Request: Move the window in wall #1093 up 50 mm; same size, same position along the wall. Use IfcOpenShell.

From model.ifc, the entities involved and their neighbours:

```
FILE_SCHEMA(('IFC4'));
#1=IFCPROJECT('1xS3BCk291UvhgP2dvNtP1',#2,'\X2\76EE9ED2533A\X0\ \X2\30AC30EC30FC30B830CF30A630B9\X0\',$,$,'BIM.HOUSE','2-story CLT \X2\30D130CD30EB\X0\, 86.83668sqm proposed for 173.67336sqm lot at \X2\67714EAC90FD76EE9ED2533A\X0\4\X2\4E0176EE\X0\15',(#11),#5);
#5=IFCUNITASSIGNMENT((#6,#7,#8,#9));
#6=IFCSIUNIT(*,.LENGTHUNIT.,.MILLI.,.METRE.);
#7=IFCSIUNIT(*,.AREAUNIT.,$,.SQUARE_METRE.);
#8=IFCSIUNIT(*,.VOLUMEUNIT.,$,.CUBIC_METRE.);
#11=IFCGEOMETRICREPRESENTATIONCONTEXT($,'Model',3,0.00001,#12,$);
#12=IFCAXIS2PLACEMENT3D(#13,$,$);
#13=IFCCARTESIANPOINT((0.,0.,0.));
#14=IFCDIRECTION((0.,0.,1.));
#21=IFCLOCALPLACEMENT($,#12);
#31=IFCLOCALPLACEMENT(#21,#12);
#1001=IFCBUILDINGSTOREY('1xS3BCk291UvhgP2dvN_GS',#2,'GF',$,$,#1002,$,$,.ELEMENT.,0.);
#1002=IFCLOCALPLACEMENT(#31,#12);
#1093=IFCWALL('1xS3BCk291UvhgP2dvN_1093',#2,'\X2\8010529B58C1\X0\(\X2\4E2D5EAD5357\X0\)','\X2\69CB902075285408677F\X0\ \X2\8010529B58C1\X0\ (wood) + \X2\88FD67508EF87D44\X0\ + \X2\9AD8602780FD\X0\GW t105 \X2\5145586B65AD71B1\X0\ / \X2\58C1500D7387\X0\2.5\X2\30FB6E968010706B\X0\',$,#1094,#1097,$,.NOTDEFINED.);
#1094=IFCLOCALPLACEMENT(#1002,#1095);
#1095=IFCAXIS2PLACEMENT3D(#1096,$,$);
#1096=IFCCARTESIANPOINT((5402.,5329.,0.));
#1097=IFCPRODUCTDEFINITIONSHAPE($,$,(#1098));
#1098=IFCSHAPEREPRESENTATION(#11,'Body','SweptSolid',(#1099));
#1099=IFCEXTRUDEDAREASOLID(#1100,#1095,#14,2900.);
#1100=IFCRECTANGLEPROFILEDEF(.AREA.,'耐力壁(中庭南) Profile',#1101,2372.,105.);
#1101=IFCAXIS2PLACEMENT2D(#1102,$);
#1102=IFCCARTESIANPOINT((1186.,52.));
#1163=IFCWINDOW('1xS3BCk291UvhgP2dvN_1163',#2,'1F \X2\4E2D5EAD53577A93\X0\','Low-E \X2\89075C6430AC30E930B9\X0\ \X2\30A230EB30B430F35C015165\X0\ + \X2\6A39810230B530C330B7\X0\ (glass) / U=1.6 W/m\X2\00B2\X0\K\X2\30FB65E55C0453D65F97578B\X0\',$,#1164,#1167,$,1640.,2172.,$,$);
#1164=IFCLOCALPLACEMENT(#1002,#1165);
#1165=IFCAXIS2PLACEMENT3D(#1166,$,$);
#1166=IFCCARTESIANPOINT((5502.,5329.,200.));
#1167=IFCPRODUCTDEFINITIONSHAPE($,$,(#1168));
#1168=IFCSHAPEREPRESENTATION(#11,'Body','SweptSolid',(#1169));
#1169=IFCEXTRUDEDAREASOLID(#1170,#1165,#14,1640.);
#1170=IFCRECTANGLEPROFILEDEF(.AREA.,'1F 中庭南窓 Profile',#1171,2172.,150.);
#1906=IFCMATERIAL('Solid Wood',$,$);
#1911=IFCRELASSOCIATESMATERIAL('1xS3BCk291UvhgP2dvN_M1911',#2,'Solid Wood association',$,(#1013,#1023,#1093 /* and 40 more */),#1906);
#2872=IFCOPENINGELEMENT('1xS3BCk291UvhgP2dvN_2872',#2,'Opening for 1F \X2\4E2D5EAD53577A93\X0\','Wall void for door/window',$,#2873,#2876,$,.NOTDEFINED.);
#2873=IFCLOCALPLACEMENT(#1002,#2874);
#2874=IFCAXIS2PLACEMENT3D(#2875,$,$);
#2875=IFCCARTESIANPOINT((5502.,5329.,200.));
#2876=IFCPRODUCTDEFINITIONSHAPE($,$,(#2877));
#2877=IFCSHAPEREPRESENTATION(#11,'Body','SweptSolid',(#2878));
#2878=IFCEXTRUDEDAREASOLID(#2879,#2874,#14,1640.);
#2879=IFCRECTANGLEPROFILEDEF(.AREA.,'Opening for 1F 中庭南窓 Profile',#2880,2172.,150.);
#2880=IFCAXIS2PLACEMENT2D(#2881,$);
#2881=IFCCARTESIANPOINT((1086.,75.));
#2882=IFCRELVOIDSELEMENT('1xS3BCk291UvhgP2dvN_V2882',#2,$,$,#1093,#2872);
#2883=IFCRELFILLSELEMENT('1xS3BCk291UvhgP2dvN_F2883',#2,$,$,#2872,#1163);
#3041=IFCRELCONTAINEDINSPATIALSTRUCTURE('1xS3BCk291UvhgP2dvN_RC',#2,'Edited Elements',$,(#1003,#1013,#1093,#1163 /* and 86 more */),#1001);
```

```python
import numpy as np
import ifcopenshell
import ifcopenshell.api.geometry
import ifcopenshell.util.placement
import ifcopenshell.util.unit

model = ifcopenshell.open("model.ifc")
unit_scale = ifcopenshell.util.unit.calculate_unit_scale(model)

window = model.by_guid("1xS3BCk291UvhgP2dvN_1163")
opening = window.FillsVoids[0].RelatingOpeningElement
dz = 50.0

shift = np.array([0.0, 0.0, dz])
# The window is not placed relative to its opening, so move both.
for product in (opening, window):
    matrix = ifcopenshell.util.placement.get_local_placement(product.ObjectPlacement)
    matrix[:3, 3] += shift
    ifcopenshell.api.geometry.edit_object_placement(model, product=product, matrix=matrix, is_si=False)

print(f"moved by {dz * unit_scale:+.3f} m")

model.write("model_rev.ifc")
```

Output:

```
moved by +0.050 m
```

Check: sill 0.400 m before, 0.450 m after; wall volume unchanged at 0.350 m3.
